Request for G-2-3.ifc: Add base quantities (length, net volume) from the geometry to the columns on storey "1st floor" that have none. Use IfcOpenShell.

First a look at what the model holds.

```python
import ifcopenshell
import ifcopenshell.util.element
import ifcopenshell.util.unit

model = ifcopenshell.open("G-2-3.ifc")
print(model.schema)
for unit_type in ("LENGTHUNIT", "AREAUNIT", "VOLUMEUNIT"):
    print(unit_type, ifcopenshell.util.unit.calculate_unit_scale(model, unit_type))
storey = next(s for s in model.by_type("IfcBuildingStorey") if s.Name == "1st floor")
columns = [e for e in ifcopenshell.util.element.get_decomposition(storey) if e.is_a("IfcColumn")]
for e in sorted(columns, key=lambda e: e.id()):
    print(e.id(), e.is_a(), e.Name, list(ifcopenshell.util.element.get_psets(e, qtos_only=True)), sep=" | ")
```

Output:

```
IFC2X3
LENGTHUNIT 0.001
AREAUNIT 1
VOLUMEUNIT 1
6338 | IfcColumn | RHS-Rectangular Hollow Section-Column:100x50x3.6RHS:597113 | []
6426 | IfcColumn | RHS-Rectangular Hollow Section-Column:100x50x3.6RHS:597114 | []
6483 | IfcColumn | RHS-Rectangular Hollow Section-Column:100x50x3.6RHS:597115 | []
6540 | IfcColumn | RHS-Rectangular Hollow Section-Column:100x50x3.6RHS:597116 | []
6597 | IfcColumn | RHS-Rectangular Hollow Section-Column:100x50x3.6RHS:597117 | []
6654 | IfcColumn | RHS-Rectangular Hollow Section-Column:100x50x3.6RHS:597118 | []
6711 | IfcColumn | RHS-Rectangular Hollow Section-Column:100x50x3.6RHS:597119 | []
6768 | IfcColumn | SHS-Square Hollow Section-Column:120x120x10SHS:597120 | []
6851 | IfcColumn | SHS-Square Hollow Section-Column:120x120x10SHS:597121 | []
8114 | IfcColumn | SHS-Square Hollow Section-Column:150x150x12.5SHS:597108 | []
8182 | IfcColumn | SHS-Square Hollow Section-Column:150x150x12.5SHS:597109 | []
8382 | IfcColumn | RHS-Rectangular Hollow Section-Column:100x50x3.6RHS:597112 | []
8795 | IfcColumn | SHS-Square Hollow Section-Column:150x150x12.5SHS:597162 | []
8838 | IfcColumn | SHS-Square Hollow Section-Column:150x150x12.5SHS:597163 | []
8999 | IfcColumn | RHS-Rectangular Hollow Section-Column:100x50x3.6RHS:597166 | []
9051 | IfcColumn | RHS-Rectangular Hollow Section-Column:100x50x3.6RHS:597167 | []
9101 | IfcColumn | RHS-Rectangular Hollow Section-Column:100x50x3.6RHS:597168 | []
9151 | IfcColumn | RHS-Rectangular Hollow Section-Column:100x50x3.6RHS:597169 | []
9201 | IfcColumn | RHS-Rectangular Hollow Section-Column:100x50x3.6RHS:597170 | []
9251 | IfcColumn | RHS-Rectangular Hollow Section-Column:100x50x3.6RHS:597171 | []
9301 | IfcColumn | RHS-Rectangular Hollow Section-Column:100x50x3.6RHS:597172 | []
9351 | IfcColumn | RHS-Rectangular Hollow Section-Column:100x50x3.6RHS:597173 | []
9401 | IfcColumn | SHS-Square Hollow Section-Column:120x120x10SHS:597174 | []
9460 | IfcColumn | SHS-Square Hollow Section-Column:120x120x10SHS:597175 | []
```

```python
import ifcopenshell
import ifcopenshell.api.pset
import ifcopenshell.geom
import ifcopenshell.util.element
import ifcopenshell.util.shape
import ifcopenshell.util.unit

model = ifcopenshell.open("G-2-3.ifc")
unit_scale = ifcopenshell.util.unit.calculate_unit_scale(model)
volume_scale = ifcopenshell.util.unit.calculate_unit_scale(model, "VOLUMEUNIT")
settings = ifcopenshell.geom.settings()

storey = next(s for s in model.by_type("IfcBuildingStorey") if s.Name == "1st floor")
columns = [e for e in ifcopenshell.util.element.get_decomposition(storey) if e.is_a("IfcColumn")]

for e in sorted(columns, key=lambda e: e.id()):
    if ifcopenshell.util.element.get_psets(e, qtos_only=True, should_inherit=False):
        continue
    # Geometry comes back in metres, in the element's own axes.
    shape = ifcopenshell.geom.create_shape(settings, e)
    values = {
        "Length": ifcopenshell.util.shape.get_z(shape.geometry) / unit_scale,
        "NetVolume": ifcopenshell.util.shape.get_volume(shape.geometry) / volume_scale,
    }
    qto = ifcopenshell.api.pset.add_qto(model, product=e, name="BaseQuantities")
    ifcopenshell.api.pset.edit_qto(model, qto=qto, properties=values)
    print(e.id(), {k: round(v, 3) for k, v in values.items()})

model.write("G-2-3_updated.ifc")
```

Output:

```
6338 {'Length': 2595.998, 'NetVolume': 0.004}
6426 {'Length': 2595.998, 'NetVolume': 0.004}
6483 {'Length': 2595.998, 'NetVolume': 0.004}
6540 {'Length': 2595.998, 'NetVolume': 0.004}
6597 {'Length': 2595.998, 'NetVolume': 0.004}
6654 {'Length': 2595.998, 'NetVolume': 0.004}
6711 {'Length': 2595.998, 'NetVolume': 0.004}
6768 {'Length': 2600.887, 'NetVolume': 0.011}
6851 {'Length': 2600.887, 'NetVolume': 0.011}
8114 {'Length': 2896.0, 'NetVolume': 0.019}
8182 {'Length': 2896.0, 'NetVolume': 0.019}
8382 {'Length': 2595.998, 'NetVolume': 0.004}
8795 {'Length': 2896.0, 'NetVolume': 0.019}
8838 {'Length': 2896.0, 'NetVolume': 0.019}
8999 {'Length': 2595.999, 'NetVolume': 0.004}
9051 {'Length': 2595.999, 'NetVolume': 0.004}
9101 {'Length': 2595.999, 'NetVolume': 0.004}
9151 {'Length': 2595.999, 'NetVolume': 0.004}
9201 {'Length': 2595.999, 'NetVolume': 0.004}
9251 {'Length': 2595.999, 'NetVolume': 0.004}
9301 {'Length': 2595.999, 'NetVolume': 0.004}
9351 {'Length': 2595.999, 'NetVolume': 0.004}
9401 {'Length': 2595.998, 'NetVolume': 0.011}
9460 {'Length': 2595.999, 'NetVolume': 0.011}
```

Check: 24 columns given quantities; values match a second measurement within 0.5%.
